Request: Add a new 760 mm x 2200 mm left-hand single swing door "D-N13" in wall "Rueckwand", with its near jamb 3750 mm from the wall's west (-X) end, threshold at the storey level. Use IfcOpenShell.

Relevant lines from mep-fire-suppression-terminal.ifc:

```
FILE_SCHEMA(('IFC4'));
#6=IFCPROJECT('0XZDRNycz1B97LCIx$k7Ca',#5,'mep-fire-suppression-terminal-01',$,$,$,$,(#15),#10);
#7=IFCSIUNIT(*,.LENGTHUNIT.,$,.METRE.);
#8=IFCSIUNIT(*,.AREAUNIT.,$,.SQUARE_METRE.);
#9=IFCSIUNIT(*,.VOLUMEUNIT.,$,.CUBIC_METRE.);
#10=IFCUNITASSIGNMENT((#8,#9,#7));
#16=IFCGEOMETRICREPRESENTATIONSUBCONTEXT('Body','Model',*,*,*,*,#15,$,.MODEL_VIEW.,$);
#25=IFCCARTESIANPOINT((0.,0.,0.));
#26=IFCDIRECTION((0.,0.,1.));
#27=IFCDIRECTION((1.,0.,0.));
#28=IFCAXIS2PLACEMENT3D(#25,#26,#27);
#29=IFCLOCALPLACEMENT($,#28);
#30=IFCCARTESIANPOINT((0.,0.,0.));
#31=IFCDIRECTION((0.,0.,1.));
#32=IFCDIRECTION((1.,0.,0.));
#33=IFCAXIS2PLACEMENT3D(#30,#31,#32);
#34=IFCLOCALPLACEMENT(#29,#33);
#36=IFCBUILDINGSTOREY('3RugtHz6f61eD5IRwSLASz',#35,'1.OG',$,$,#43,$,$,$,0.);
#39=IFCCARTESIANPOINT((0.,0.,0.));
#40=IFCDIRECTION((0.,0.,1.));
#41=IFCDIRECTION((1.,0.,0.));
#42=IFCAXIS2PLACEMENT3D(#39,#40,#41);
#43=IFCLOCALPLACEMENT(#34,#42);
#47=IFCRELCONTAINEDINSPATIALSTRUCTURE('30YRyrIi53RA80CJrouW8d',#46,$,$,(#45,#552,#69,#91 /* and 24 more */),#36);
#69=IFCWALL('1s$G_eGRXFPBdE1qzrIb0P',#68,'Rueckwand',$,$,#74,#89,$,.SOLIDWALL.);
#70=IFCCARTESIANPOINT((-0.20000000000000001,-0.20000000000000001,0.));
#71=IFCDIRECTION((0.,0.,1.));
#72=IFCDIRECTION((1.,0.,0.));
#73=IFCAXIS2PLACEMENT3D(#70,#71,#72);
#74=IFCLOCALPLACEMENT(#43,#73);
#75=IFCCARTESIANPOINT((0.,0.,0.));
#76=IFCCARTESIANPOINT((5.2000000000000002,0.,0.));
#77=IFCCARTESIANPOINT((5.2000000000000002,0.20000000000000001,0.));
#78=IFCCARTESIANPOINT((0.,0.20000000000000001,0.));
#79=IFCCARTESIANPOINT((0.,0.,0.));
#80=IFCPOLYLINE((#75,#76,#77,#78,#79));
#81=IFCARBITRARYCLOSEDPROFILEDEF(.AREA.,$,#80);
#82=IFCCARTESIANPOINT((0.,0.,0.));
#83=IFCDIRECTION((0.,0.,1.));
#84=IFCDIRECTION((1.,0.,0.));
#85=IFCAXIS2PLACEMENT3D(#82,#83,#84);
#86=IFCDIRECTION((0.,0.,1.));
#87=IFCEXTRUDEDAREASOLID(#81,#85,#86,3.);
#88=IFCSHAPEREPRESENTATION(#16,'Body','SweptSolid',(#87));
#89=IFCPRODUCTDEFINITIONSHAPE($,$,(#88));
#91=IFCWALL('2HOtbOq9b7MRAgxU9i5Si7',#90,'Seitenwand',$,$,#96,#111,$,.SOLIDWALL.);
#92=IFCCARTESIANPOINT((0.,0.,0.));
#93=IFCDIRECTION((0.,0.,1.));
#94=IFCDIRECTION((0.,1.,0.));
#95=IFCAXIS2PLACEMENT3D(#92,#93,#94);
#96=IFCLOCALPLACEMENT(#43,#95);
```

```python
import numpy as np
import ifcopenshell
import ifcopenshell.api.feature
import ifcopenshell.api.geometry
import ifcopenshell.api.root
import ifcopenshell.api.spatial
import ifcopenshell.geom
import ifcopenshell.util.element
import ifcopenshell.util.placement
import ifcopenshell.util.representation
import ifcopenshell.util.shape
import ifcopenshell.util.unit

model = ifcopenshell.open("mep-fire-suppression-terminal.ifc")
unit_scale = ifcopenshell.util.unit.calculate_unit_scale(model)
settings = ifcopenshell.geom.settings()


def volume(element):
    """Net volume in cubic metres, openings subtracted."""
    shape = ifcopenshell.geom.create_shape(settings, element)
    return ifcopenshell.util.shape.get_volume(shape.geometry)


wall = model.by_guid("1s$G_eGRXFPBdE1qzrIb0P")
storey = ifcopenshell.util.element.get_container(wall, ifc_class="IfcBuildingStorey")
context = ifcopenshell.util.representation.get_context(model, "Model", "Body", "MODEL_VIEW")
before = volume(wall)

width, height, from_end, sill = 0.76, 2.2, 3.75, 0.0  # metres

# The wall runs along its own X axis, and the end named is its -X end.
wall_shape = ifcopenshell.geom.create_shape(settings, wall)
x, y, z = ifcopenshell.util.shape.get_vertices(wall_shape.geometry).T
start = x.min() + from_end
face, thickness = float(y.min()), float(y.max() - y.min())
wall_matrix = ifcopenshell.util.placement.get_local_placement(wall.ObjectPlacement)
level = ifcopenshell.util.placement.get_local_placement(storey.ObjectPlacement)[2, 3]


def in_wall(x, y):
    """Placement at x, y metres in the wall's axes, at sill height."""
    matrix = wall_matrix.copy()
    matrix[:, 3] = wall_matrix @ np.array([x / unit_scale, y / unit_scale, 0.0, 1.0])
    matrix[2, 3] = level + sill / unit_scale
    return matrix


# Opening: a box that overshoots both wall faces by 50 mm.
opening = ifcopenshell.api.root.create_entity(model, ifc_class="IfcOpeningElement", predefined_type="OPENING")
box = ifcopenshell.api.geometry.add_wall_representation(
    model, context=context, length=width, height=height, thickness=thickness + 0.1
)
ifcopenshell.api.geometry.assign_representation(model, product=opening, representation=box)
ifcopenshell.api.geometry.edit_object_placement(model, product=opening, matrix=in_wall(start, face - 0.05), is_si=False)
ifcopenshell.api.feature.add_feature(model, feature=opening, element=wall)

door = ifcopenshell.api.root.create_entity(model, ifc_class="IfcDoor", name="D-N13", predefined_type="DOOR")
door.OverallWidth, door.OverallHeight = width / unit_scale, height / unit_scale
door.OperationType = "SINGLE_SWING_LEFT"
body = ifcopenshell.api.geometry.add_door_representation(
    model,
    context=context,
    overall_width=door.OverallWidth,
    overall_height=door.OverallHeight,
    operation_type="SINGLE_SWING_LEFT",
    lining_properties={"LiningDepth": thickness / unit_scale, "ThresholdDepth": thickness / unit_scale},
)
ifcopenshell.api.geometry.assign_representation(model, product=door, representation=body)
ifcopenshell.api.spatial.assign_container(model, products=[door], relating_structure=storey)
ifcopenshell.api.feature.add_filling(model, opening=opening, element=door)

# The lining spans the wall, so the door starts at the wall face.
ifcopenshell.api.geometry.edit_object_placement(model, product=door, matrix=in_wall(start, face), is_si=False)

after = volume(wall)

print(f"wall volume {before:.3f} -> {after:.3f} m3")

model.write("mep-fire-suppression-terminal-out.ifc")
```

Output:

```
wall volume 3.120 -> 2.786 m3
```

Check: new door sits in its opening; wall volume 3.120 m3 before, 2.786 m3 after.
